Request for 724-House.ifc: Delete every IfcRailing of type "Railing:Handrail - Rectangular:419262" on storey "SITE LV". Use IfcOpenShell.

First a look at what the model holds.

```python
import ifcopenshell
import ifcopenshell.util.element

model = ifcopenshell.open("724-House.ifc")
print(model.schema)
storey = next(s for s in model.by_type("IfcBuildingStorey") if s.Name == "SITE LV")
railings = [e for e in ifcopenshell.util.element.get_decomposition(storey) if e.is_a("IfcRailing")]
seen = {}
for e in railings:
    element_type = ifcopenshell.util.element.get_type(e)
    name = element_type.Name if element_type not in (None, e) else None
    seen[name] = seen.get(name, 0) + 1
for name, count in sorted(seen.items(), key=str):
    print(count, "x", name)
```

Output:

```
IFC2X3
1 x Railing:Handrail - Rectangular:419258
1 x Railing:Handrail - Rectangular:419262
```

```python
import ifcopenshell
import ifcopenshell.api.root
import ifcopenshell.util.element

model = ifcopenshell.open("724-House.ifc")

storey = next(s for s in model.by_type("IfcBuildingStorey") if s.Name == "SITE LV")
railings = [e for e in ifcopenshell.util.element.get_decomposition(storey) if e.is_a("IfcRailing")]
targets = [e for e in railings if (t := ifcopenshell.util.element.get_type(e)) not in (None, e) and t.Name == "Railing:Handrail - Rectangular:419262"]

for e in targets:
    ifcopenshell.api.root.remove_product(model, product=e)
print(len(targets), "removed")

model.write("724-House_v2.ifc")
```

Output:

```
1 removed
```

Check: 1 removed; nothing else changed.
